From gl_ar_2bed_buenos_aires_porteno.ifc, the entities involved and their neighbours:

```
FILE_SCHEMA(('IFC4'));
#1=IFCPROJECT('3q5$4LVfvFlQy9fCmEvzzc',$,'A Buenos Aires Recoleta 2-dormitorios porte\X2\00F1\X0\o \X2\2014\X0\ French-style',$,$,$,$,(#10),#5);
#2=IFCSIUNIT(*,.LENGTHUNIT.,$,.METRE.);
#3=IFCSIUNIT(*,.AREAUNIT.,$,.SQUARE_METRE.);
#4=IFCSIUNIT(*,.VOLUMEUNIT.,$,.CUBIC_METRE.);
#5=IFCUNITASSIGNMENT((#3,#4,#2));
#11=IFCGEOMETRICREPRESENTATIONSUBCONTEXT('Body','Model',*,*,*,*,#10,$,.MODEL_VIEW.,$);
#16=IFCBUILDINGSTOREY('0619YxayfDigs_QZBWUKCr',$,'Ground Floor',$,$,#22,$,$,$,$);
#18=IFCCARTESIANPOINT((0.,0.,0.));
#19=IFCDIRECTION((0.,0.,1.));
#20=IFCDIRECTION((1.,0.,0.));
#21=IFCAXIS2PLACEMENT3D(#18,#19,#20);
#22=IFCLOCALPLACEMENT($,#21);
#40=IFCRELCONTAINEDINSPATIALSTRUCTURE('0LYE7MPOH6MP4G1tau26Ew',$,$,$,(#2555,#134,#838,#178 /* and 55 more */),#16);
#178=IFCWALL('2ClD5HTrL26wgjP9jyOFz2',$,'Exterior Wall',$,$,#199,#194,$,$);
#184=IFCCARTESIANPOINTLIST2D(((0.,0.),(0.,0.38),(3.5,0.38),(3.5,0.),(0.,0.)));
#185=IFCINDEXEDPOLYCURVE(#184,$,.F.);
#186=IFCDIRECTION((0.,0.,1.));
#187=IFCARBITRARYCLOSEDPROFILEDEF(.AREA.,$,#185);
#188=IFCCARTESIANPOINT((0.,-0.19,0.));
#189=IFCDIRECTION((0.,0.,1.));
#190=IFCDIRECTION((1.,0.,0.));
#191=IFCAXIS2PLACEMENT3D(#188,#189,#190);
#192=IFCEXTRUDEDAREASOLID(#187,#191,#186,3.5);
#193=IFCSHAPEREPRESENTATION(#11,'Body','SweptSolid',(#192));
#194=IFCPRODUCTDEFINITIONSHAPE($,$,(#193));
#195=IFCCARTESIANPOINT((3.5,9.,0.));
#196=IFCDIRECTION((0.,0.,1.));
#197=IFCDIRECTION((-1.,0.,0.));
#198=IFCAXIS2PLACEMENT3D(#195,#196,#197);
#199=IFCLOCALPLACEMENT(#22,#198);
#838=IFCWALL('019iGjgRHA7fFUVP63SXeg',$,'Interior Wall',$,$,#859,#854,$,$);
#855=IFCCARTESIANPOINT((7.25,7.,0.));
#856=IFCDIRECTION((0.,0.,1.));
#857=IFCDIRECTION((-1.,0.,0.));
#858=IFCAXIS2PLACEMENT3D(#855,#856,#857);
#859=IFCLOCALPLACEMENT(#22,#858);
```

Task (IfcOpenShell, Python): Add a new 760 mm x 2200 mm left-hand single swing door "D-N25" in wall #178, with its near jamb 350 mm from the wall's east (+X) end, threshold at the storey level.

```python
import numpy as np
import ifcopenshell
import ifcopenshell.api.feature
import ifcopenshell.api.geometry
import ifcopenshell.api.root
import ifcopenshell.api.spatial
import ifcopenshell.geom
import ifcopenshell.util.element
import ifcopenshell.util.placement
import ifcopenshell.util.representation
import ifcopenshell.util.shape
import ifcopenshell.util.unit

model = ifcopenshell.open("gl_ar_2bed_buenos_aires_porteno.ifc")
unit_scale = ifcopenshell.util.unit.calculate_unit_scale(model)
settings = ifcopenshell.geom.settings()


def volume(element):
    """Net volume in cubic metres, openings subtracted."""
    shape = ifcopenshell.geom.create_shape(settings, element)
    return ifcopenshell.util.shape.get_volume(shape.geometry)


wall = model.by_guid("2ClD5HTrL26wgjP9jyOFz2")
storey = ifcopenshell.util.element.get_container(wall, ifc_class="IfcBuildingStorey")
context = ifcopenshell.util.representation.get_context(model, "Model", "Body", "MODEL_VIEW")
before = volume(wall)

width, height, from_end, sill = 0.76, 2.2, 0.35, 0.0  # metres

# The wall runs along its own X axis, and the end named is its -X end.
wall_shape = ifcopenshell.geom.create_shape(settings, wall)
x, y, z = ifcopenshell.util.shape.get_vertices(wall_shape.geometry).T
start = x.min() + from_end
face, thickness = float(y.min()), float(y.max() - y.min())
wall_matrix = ifcopenshell.util.placement.get_local_placement(wall.ObjectPlacement)
level = ifcopenshell.util.placement.get_local_placement(storey.ObjectPlacement)[2, 3]


def in_wall(x, y):
    """Placement at x, y metres in the wall's axes, at sill height."""
    matrix = wall_matrix.copy()
    matrix[:, 3] = wall_matrix @ np.array([x / unit_scale, y / unit_scale, 0.0, 1.0])
    matrix[2, 3] = level + sill / unit_scale
    return matrix


# Opening: a box that overshoots both wall faces by 50 mm.
opening = ifcopenshell.api.root.create_entity(model, ifc_class="IfcOpeningElement", predefined_type="OPENING")
box = ifcopenshell.api.geometry.add_wall_representation(
    model, context=context, length=width, height=height, thickness=thickness + 0.1
)
ifcopenshell.api.geometry.assign_representation(model, product=opening, representation=box)
ifcopenshell.api.geometry.edit_object_placement(model, product=opening, matrix=in_wall(start, face - 0.05), is_si=False)
ifcopenshell.api.feature.add_feature(model, feature=opening, element=wall)

door = ifcopenshell.api.root.create_entity(model, ifc_class="IfcDoor", name="D-N25", predefined_type="DOOR")
door.OverallWidth, door.OverallHeight = width / unit_scale, height / unit_scale
door.OperationType = "SINGLE_SWING_LEFT"
body = ifcopenshell.api.geometry.add_door_representation(
    model,
    context=context,
    overall_width=door.OverallWidth,
    overall_height=door.OverallHeight,
    operation_type="SINGLE_SWING_LEFT",
    lining_properties={"LiningDepth": thickness / unit_scale, "ThresholdDepth": thickness / unit_scale},
)
ifcopenshell.api.geometry.assign_representation(model, product=door, representation=body)
ifcopenshell.api.spatial.assign_container(model, products=[door], relating_structure=storey)
ifcopenshell.api.feature.add_filling(model, opening=opening, element=door)

# The lining spans the wall, so the door starts at the wall face.
ifcopenshell.api.geometry.edit_object_placement(model, product=door, matrix=in_wall(start, face), is_si=False)

after = volume(wall)

print(f"wall volume {before:.3f} -> {after:.3f} m3")

model.write("gl_ar_2bed_buenos_aires_porteno_updated.ifc")
```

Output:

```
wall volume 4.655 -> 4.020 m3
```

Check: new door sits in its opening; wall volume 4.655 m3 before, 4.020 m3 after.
